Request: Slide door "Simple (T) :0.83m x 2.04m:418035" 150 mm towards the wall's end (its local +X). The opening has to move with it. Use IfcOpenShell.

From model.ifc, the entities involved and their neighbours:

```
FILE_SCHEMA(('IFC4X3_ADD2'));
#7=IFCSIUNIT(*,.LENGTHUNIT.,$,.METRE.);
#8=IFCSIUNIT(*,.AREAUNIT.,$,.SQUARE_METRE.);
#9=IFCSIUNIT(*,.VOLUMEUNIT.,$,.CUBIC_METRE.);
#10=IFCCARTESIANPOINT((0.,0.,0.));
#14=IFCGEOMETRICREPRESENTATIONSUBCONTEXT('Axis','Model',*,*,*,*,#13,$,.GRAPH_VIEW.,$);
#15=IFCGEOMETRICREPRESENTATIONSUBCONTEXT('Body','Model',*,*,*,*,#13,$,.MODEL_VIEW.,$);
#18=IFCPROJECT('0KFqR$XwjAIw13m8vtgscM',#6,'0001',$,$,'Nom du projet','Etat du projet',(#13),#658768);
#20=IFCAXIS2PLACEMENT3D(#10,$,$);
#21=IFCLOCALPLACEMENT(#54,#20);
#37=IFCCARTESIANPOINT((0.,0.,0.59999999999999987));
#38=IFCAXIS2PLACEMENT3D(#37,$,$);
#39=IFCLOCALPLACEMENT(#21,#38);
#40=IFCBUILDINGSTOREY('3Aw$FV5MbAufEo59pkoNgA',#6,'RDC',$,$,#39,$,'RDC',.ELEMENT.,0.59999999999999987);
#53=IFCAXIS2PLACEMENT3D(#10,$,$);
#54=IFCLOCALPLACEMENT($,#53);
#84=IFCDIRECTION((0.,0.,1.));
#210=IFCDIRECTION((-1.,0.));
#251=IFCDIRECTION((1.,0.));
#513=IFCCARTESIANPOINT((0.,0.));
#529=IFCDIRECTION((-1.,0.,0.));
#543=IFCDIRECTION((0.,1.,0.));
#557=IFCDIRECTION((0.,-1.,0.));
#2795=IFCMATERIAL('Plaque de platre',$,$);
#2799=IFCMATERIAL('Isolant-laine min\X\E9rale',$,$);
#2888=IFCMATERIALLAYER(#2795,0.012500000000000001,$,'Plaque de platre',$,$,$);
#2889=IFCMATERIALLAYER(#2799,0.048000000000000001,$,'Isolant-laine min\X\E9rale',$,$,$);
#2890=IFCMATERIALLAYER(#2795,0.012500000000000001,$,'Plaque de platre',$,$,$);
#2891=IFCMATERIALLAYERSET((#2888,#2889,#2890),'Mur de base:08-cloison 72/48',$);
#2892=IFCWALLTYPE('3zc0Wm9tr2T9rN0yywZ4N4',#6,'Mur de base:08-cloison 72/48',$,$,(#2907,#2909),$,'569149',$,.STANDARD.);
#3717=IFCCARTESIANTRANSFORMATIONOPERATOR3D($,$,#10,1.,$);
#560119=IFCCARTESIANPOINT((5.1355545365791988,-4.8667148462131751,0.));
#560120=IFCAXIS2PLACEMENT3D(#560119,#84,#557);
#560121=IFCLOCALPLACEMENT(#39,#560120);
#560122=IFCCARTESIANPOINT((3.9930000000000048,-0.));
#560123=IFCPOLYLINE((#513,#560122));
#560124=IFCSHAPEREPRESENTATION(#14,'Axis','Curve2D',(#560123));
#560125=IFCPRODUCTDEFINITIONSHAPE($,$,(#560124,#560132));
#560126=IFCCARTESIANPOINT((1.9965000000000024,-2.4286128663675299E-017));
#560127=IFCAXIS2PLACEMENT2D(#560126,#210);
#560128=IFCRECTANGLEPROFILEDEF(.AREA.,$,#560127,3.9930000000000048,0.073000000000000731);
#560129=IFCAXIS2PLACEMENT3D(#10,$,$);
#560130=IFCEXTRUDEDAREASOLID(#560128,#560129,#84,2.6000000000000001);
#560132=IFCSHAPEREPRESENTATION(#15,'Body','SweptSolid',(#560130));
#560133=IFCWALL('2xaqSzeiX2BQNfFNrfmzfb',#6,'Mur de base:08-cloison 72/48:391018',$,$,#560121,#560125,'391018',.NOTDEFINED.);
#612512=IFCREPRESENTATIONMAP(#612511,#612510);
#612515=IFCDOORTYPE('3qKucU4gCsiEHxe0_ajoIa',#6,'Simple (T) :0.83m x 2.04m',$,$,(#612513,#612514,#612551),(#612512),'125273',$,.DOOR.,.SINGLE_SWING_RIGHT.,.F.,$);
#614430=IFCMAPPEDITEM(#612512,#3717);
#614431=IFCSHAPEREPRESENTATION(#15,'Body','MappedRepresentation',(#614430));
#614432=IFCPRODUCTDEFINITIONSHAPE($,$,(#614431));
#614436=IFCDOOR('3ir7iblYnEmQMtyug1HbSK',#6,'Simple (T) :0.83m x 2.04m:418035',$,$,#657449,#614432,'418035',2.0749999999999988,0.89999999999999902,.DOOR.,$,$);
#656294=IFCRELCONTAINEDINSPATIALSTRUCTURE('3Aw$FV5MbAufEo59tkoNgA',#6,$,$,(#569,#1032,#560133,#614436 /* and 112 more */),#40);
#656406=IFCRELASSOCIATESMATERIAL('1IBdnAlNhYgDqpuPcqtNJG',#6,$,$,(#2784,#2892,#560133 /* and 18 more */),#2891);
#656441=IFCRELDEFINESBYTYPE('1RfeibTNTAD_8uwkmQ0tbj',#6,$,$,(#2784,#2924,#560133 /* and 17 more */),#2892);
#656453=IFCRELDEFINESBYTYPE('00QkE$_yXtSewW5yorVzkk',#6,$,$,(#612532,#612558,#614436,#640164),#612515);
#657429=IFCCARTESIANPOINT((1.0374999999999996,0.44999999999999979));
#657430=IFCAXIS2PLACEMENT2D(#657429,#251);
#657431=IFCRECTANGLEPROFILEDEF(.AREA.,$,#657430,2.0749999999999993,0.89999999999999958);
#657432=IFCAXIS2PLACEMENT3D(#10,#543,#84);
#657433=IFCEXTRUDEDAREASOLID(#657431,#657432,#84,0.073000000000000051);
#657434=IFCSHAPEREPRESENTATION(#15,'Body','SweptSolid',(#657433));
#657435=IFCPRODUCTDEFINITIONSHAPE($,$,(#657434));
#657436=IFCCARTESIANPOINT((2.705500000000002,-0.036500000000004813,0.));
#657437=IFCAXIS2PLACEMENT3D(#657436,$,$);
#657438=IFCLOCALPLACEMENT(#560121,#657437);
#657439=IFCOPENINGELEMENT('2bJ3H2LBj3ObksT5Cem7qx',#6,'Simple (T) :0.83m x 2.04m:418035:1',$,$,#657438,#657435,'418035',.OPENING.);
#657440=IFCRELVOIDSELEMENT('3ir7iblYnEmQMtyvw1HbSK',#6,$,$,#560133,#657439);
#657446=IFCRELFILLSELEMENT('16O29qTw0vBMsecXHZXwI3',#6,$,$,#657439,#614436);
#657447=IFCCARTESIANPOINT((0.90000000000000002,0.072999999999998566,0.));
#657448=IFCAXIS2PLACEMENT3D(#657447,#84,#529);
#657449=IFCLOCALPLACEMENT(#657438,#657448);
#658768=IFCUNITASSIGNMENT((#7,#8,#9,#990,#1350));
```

```python
import ifcopenshell
import ifcopenshell.api.geometry
import ifcopenshell.util.placement
import ifcopenshell.util.unit

model = ifcopenshell.open("model.ifc")
unit_scale = ifcopenshell.util.unit.calculate_unit_scale(model)

door = model.by_guid("3ir7iblYnEmQMtyug1HbSK")
opening = door.FillsVoids[0].RelatingOpeningElement
wall = opening.VoidsElements[0].RelatingBuildingElement

wall_matrix = ifcopenshell.util.placement.get_local_placement(wall.ObjectPlacement)
shift = wall_matrix[:3, 0] * 0.15 / unit_scale
before = ifcopenshell.util.placement.get_local_placement(door.ObjectPlacement)[:3, 3].copy()

# The door is placed relative to its opening, so it follows when the opening moves.
matrix = ifcopenshell.util.placement.get_local_placement(opening.ObjectPlacement)
matrix[:3, 3] += shift
ifcopenshell.api.geometry.edit_object_placement(
    model, product=opening, matrix=matrix, is_si=False, should_transform_children=True
)

after = ifcopenshell.util.placement.get_local_placement(door.ObjectPlacement)[:3, 3]
print("door moved by", (after - before).round(3) + 0.0)

model.write("model_updated.ifc")
```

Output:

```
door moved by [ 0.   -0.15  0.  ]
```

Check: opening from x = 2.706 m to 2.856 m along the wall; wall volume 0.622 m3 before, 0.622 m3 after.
